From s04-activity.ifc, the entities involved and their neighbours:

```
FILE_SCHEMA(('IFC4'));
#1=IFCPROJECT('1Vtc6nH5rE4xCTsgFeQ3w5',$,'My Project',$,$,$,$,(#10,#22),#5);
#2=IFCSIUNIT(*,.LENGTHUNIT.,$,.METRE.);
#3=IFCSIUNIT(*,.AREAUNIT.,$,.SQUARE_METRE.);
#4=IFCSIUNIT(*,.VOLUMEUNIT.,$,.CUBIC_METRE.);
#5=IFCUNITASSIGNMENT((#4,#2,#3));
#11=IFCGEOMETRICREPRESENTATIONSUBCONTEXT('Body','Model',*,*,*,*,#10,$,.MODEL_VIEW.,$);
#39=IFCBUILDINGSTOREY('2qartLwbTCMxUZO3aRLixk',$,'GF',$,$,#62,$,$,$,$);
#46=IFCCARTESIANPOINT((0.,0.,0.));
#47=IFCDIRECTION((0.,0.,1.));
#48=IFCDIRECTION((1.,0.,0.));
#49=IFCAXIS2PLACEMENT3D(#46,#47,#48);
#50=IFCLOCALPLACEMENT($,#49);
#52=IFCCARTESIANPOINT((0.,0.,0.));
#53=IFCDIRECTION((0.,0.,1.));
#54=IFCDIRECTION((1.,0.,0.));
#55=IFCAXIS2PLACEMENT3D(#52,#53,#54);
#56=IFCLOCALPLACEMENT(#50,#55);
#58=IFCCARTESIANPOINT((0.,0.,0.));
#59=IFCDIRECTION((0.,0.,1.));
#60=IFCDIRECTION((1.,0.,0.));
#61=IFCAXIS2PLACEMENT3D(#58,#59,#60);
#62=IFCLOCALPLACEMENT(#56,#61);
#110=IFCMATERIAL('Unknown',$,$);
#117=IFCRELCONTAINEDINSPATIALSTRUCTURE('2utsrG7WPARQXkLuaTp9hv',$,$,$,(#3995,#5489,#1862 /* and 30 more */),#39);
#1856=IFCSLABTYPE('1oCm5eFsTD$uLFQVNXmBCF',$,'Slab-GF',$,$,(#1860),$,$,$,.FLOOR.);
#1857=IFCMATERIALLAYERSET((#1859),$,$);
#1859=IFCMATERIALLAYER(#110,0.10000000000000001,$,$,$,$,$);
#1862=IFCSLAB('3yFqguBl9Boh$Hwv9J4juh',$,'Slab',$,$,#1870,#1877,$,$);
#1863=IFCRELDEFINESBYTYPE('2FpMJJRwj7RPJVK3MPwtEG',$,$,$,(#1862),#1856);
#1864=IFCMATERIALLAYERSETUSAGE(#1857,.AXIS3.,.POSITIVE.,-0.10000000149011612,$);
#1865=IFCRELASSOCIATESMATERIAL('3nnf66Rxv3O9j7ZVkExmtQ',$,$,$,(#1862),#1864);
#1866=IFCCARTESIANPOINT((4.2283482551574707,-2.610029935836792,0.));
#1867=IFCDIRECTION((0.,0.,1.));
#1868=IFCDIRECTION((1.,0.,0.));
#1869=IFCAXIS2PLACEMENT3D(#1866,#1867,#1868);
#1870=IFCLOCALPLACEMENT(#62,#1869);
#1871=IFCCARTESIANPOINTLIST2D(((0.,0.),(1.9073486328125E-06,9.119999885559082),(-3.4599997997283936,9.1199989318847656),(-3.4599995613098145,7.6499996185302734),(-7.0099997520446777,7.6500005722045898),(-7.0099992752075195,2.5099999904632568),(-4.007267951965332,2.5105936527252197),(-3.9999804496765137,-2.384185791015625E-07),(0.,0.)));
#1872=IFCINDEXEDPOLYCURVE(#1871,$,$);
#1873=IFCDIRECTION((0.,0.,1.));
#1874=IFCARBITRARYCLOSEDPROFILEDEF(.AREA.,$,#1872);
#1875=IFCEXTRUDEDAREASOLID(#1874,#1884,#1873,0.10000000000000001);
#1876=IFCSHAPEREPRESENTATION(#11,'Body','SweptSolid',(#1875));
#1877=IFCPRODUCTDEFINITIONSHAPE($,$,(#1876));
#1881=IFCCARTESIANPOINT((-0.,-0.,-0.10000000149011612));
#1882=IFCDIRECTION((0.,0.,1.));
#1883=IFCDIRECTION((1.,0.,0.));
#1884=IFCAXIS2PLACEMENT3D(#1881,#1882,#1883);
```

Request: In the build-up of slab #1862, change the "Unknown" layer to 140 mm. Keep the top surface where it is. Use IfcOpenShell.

```python
import ifcopenshell
import ifcopenshell.util.element
import ifcopenshell.util.representation

model = ifcopenshell.open("s04-activity.ifc")

layer_set = model.by_id(1857)
layer = next(l for l in layer_set.MaterialLayers if l.Material and l.Material.Name == "Unknown")
change = 0.14 - layer.LayerThickness
layer.LayerThickness += change

# Geometry does not follow the layer set by itself.
slabs = [e for e in ifcopenshell.util.element.get_elements_by_material(model, layer_set) if e.is_a("IfcSlab")]
for slab in sorted(slabs, key=lambda e: e.id()):
    body = ifcopenshell.util.representation.get_representation(slab, "Model", "Body")
    solid = body.Items[0]
    old_depth = solid.Depth
    solid.Depth += change
    # Extruded upwards: lower the start of the extrusion so the top stays.
    x, y, z = solid.Position.Location.Coordinates
    solid.Position.Location = model.createIfcCartesianPoint((x, y, z - change))
    print(slab.id(), f"{old_depth:g} -> {solid.Depth:g}")

# The layers are counted up from the underside, which has moved.
for usage in {ifcopenshell.util.element.get_material(slab) for slab in slabs}:
    usage.OffsetFromReferenceLine -= change

model.write("s04-activity_updated.ifc")
```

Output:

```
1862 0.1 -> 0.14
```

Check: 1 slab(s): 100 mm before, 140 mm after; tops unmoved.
